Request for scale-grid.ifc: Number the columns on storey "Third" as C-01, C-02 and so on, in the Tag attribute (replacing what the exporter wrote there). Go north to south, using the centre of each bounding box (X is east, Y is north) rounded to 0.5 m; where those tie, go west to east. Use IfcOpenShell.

First a look at what the model holds.

```python
import ifcopenshell
import ifcopenshell.util.element
import ifcopenshell.util.placement

model = ifcopenshell.open("scale-grid.ifc")
print(model.schema)
storey = next(s for s in model.by_type("IfcBuildingStorey") if s.Name == "Third")
columns = [e for e in ifcopenshell.util.element.get_decomposition(storey) if e.is_a("IfcColumn")]
for e in sorted(columns, key=lambda e: e.id()):
    origin = ifcopenshell.util.placement.get_local_placement(e.ObjectPlacement)[:3, 3]
    print(e.id(), e.Tag, e.Name, origin.round(2) + 0.0, sep=" | ")
```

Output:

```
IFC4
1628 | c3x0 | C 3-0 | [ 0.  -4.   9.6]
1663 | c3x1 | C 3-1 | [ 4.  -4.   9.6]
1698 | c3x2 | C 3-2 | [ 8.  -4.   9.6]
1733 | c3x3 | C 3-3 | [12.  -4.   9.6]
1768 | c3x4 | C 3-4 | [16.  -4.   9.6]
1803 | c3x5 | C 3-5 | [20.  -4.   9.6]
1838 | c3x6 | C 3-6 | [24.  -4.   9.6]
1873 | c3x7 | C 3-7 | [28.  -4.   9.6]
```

```python
import ifcopenshell
import ifcopenshell.geom
import ifcopenshell.util.element
import ifcopenshell.util.shape

model = ifcopenshell.open("scale-grid.ifc")
settings = ifcopenshell.geom.settings()
settings.set("use-world-coords", True)


def centre(element):
    shape = ifcopenshell.geom.create_shape(settings, element)
    return ifcopenshell.util.shape.get_bbox_centroid(shape.geometry)


storey = next(s for s in model.by_type("IfcBuildingStorey") if s.Name == "Third")
columns = [e for e in ifcopenshell.util.element.get_decomposition(storey) if e.is_a("IfcColumn")]

# Insertion points can sit at a corner or the storey origin, so sort by the geometry (in metres).
centres = {e: centre(e) for e in columns}
columns.sort(key=lambda e: (-round(centres[e][1] / 0.5), centres[e][0]))

for i, e in enumerate(columns, start=1):
    number = f"C-{i:02d}"
    e.Tag = number
    print(e.id(), number)

model.write("scale-grid_v2.ifc")
```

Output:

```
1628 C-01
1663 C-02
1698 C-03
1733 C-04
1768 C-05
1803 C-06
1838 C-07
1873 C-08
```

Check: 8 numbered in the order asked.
